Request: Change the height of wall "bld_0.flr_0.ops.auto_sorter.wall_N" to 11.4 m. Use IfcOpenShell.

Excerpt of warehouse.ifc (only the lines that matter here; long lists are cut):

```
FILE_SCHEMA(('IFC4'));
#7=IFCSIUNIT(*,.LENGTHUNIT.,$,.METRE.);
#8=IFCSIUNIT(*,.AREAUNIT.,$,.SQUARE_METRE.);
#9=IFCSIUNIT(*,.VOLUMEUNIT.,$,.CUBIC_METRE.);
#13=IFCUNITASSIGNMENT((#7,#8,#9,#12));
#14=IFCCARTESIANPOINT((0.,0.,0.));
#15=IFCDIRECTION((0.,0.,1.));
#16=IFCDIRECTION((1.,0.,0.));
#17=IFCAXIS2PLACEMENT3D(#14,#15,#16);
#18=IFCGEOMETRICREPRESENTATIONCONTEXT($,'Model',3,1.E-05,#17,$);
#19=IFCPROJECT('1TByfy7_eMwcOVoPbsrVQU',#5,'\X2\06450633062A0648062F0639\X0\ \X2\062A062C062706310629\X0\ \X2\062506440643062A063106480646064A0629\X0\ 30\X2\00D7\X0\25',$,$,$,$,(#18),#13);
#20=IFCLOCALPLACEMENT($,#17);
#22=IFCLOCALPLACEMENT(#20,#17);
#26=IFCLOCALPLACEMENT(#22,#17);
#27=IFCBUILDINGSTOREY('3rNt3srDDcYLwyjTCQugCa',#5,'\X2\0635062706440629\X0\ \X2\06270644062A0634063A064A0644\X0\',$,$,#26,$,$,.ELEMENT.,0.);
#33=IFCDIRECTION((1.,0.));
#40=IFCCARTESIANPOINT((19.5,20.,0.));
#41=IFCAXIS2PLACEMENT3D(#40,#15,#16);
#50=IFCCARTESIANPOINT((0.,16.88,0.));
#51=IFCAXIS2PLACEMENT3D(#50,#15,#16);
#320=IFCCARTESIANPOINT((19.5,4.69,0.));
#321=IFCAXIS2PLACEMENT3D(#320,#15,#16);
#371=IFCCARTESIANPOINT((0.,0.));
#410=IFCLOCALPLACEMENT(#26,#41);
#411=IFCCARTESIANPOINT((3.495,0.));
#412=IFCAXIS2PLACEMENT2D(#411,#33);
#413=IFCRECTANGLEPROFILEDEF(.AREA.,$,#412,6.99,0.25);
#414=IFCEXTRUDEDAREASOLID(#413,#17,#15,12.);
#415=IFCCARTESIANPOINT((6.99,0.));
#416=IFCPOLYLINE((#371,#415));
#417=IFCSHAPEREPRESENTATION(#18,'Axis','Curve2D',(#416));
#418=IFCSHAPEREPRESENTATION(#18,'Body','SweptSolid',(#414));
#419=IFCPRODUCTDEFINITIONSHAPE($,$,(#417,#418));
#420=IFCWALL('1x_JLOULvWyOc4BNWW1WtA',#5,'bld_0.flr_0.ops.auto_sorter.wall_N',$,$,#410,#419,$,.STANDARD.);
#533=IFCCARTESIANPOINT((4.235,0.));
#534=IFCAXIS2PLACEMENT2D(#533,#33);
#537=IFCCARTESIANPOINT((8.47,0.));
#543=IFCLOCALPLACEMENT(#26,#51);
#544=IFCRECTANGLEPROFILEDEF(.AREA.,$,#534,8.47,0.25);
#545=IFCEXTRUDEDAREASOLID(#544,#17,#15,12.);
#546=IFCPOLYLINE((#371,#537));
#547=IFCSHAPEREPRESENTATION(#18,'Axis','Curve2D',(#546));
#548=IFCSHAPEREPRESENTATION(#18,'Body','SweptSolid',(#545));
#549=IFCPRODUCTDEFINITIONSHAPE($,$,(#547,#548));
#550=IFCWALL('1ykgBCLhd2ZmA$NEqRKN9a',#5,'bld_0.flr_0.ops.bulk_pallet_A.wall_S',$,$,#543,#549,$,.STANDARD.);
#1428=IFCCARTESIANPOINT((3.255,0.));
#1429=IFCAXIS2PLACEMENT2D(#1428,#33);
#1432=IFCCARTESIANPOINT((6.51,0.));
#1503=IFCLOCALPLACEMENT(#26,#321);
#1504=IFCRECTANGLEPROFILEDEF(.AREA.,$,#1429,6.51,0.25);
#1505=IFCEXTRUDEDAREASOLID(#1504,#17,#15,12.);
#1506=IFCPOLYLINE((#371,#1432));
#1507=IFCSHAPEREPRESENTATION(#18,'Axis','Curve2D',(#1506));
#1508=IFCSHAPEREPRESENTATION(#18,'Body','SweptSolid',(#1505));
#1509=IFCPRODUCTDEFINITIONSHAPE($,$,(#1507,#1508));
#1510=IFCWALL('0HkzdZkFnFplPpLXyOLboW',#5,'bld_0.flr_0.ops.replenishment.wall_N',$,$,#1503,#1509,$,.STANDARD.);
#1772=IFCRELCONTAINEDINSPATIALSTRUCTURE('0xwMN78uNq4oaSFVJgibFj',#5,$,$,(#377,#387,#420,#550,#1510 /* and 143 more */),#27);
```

```python
import ifcopenshell
import ifcopenshell.geom
import ifcopenshell.util.shape
import ifcopenshell.util.unit

model = ifcopenshell.open("warehouse.ifc")
unit_scale = ifcopenshell.util.unit.calculate_unit_scale(model)
settings = ifcopenshell.geom.settings()


def volume(element):
    """Net volume in cubic metres, openings subtracted."""
    shape = ifcopenshell.geom.create_shape(settings, element)
    return ifcopenshell.util.shape.get_volume(shape.geometry)


wall = model.by_id(420)
before = volume(wall)

body = next(r for r in wall.Representation.Representations if r.RepresentationIdentifier == "Body")
solid = body.Items[0]
old_height = solid.Depth
solid.Depth = 11.4 / unit_scale
after = volume(wall)

print(f"height {old_height:g} -> {solid.Depth:g}, volume {before:.3f} -> {after:.3f} m3")

model.write("warehouse_v2.ifc")
```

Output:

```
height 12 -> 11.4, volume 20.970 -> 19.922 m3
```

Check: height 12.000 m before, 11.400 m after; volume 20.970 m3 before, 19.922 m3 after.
